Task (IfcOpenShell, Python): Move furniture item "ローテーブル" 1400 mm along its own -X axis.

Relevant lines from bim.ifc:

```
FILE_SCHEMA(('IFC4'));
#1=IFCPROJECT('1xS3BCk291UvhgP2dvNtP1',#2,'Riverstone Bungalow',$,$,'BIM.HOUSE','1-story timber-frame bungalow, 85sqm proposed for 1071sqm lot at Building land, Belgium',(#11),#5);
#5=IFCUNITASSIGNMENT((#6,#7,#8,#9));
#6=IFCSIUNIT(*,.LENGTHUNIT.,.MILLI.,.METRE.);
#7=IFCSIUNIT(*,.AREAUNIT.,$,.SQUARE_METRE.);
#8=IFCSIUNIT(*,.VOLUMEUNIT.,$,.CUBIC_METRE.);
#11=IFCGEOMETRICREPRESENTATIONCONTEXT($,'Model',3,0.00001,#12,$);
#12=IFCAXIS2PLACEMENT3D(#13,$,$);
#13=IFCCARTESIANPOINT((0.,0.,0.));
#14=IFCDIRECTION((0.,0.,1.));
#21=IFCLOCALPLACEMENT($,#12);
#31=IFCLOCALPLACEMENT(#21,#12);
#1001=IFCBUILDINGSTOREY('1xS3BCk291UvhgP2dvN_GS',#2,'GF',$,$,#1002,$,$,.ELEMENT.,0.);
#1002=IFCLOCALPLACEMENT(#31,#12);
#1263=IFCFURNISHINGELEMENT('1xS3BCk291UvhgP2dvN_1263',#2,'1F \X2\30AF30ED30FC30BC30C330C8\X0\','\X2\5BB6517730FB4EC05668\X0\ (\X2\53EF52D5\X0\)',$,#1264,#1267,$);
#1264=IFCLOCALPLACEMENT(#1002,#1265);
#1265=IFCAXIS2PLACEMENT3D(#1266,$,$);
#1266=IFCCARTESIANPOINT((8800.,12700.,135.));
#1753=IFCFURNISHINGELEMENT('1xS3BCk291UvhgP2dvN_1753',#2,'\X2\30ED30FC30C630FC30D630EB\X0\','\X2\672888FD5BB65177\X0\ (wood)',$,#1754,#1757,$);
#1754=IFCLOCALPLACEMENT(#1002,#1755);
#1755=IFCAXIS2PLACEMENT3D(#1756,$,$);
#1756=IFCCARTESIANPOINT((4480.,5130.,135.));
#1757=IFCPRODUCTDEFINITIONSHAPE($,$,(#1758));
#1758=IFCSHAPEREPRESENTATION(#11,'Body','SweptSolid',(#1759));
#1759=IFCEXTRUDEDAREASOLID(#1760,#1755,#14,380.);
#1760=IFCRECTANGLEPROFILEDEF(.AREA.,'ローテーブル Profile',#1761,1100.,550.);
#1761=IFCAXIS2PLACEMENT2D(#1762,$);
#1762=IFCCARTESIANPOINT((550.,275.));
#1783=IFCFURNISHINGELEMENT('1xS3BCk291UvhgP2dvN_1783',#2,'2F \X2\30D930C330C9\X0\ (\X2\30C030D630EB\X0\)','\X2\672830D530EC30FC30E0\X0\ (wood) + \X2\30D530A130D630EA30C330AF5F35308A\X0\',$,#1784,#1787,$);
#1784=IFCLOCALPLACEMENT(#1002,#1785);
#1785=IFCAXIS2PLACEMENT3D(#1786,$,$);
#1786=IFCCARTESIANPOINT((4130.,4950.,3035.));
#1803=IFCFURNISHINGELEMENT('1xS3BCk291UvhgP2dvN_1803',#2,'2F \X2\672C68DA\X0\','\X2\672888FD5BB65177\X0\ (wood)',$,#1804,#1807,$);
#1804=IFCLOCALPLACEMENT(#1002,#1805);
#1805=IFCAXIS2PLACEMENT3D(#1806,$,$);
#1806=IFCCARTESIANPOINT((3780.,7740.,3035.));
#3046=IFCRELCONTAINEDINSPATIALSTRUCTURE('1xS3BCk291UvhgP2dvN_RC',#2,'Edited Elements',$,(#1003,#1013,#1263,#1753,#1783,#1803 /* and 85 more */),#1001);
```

```python
import ifcopenshell
import ifcopenshell.api.geometry
import ifcopenshell.util.placement
import ifcopenshell.util.unit

model = ifcopenshell.open("bim.ifc")
unit_scale = ifcopenshell.util.unit.calculate_unit_scale(model)

item = model.by_id(1753)
matrix = ifcopenshell.util.placement.get_local_placement(item.ObjectPlacement)
matrix[:3, 3] -= matrix[:3, 0] * 1.4 / unit_scale
ifcopenshell.api.geometry.edit_object_placement(model, product=item, matrix=matrix, is_si=False)

print(ifcopenshell.util.placement.get_local_placement(item.ObjectPlacement).round(3) + 0.0)

model.write("bim_v2.ifc")
```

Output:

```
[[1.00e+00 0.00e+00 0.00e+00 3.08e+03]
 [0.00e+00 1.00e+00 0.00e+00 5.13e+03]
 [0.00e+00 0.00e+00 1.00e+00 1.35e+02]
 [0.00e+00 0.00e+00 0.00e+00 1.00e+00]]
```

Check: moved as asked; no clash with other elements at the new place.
